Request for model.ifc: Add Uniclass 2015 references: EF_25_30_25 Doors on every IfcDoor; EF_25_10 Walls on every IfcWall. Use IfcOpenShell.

First a look at what the model holds.

```python
import ifcopenshell

model = ifcopenshell.open("model.ifc")
print(model.schema)
print("classifications:", [c.Name for c in model.by_type("IfcClassification")])
for ifc_class in ("IfcDoor", "IfcRoof", "IfcStair", "IfcWall", "IfcWindow"):
    print(ifc_class, len(model.by_type(ifc_class)))
```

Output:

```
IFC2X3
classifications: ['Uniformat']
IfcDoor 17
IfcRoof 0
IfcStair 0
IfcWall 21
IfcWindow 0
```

```python
import ifcopenshell
import ifcopenshell.api.classification

model = ifcopenshell.open("model.ifc")

# IFC2X3 requires Source and Edition and has no link from the project to the system.
system = model.create_entity("IfcClassification", Source="NBS", Edition="2015", Name="Uniclass 2015")

codes = {
    "IfcDoor": ("EF_25_30_25", "Doors"),
    "IfcWall": ("EF_25_10", "Walls"),
}
for ifc_class, (code, name) in codes.items():
    products = model.by_type(ifc_class)
    ifcopenshell.api.classification.add_reference(
        model, products=products, classification=system, identification=code, name=name
    )
    print(code, len(products))

model.write("model_updated.ifc")
```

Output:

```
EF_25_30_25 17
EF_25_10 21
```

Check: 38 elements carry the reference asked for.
